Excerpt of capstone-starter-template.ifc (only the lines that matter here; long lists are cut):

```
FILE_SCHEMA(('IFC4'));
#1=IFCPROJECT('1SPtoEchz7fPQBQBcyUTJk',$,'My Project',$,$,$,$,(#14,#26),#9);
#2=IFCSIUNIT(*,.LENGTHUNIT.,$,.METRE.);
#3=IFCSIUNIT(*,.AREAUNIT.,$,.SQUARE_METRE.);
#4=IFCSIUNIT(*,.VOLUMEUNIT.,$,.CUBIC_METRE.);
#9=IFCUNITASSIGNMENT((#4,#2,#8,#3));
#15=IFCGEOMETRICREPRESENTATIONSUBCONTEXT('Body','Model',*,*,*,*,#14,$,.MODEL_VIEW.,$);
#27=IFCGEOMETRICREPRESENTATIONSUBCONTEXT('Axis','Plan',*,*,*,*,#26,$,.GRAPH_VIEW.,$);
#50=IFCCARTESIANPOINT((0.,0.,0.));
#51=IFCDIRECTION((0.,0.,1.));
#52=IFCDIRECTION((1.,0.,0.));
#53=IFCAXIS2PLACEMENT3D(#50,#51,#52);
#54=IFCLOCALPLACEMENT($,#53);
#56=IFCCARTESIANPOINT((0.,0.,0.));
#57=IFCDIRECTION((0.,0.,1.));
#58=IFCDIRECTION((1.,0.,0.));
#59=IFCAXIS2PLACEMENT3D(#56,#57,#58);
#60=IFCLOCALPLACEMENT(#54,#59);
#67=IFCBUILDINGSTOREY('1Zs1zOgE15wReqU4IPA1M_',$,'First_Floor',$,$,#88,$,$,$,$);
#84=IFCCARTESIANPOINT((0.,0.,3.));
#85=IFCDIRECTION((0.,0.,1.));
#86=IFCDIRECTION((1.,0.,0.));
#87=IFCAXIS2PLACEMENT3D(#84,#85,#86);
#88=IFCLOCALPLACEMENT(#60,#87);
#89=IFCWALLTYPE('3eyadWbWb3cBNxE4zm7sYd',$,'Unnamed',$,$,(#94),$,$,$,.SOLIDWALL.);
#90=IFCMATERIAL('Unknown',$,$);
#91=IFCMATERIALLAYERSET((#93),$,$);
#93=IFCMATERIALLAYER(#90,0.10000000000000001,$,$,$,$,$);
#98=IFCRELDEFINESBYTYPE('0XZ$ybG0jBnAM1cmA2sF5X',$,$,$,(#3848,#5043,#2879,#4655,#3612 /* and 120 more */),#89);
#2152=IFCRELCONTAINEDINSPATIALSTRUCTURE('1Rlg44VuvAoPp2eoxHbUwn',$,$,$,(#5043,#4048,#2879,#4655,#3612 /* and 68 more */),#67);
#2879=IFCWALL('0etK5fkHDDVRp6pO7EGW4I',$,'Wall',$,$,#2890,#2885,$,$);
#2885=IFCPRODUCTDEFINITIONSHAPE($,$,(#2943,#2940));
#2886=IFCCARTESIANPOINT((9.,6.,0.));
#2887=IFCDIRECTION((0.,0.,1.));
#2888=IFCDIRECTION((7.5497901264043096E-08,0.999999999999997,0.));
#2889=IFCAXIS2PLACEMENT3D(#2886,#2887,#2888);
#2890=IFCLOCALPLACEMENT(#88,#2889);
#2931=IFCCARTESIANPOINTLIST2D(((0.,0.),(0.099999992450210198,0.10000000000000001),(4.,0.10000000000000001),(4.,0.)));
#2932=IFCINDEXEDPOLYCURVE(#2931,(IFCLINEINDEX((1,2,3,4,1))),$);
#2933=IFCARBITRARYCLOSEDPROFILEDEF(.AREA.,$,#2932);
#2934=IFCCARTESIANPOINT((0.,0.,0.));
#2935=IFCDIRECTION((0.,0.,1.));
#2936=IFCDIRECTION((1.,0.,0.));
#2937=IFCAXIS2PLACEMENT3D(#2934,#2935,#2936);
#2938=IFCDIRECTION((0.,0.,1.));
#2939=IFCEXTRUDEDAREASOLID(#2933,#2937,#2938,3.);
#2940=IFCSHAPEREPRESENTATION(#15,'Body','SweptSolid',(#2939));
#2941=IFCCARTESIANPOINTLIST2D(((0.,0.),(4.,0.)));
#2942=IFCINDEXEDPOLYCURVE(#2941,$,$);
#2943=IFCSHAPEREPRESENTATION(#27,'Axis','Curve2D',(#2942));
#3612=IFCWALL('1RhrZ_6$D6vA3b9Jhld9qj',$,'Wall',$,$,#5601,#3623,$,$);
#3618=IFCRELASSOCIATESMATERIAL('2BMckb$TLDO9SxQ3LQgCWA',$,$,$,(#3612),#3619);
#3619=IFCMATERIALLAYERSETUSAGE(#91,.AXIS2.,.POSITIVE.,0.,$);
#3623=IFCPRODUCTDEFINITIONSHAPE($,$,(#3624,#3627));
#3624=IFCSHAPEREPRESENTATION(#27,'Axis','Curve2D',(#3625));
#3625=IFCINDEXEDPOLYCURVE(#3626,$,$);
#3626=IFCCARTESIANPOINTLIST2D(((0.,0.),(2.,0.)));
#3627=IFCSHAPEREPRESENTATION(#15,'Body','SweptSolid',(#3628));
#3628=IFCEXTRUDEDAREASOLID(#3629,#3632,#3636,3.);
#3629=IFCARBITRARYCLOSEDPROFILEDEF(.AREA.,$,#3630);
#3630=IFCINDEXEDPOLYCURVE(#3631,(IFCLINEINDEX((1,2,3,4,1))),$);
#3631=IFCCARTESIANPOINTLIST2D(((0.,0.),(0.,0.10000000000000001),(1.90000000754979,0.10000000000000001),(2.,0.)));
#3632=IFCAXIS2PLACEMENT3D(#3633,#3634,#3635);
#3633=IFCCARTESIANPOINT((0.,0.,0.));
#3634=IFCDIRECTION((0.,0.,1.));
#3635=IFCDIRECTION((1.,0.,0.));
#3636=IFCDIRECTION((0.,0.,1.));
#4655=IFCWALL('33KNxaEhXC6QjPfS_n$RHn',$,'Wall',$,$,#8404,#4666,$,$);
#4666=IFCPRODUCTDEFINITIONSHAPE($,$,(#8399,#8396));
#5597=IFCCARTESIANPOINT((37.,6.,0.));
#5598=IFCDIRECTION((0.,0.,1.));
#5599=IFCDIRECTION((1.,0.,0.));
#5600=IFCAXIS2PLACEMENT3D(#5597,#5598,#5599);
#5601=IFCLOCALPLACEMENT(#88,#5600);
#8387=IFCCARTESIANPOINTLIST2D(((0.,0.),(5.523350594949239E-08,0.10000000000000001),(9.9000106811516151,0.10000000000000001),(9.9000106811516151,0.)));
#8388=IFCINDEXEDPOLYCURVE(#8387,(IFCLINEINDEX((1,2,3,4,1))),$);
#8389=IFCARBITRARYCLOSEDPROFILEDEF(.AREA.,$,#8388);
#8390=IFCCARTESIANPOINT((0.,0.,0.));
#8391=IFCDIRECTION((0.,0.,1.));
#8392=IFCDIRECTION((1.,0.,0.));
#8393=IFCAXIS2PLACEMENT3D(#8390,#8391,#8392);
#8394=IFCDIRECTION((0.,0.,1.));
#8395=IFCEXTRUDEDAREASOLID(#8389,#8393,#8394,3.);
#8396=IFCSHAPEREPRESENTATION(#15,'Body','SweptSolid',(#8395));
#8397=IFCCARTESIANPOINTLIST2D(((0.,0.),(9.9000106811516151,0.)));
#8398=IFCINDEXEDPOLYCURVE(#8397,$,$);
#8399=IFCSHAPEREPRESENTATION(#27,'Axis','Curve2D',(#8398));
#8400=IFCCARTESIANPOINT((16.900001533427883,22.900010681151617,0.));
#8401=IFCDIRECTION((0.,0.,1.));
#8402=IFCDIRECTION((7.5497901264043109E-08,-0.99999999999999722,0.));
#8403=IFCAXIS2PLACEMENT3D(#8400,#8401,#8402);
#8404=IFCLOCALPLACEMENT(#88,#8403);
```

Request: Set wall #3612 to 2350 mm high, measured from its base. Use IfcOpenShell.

```python
import ifcopenshell
import ifcopenshell.geom
import ifcopenshell.util.representation
import ifcopenshell.util.shape
import ifcopenshell.util.unit

model = ifcopenshell.open("capstone-starter-template.ifc")
unit_scale = ifcopenshell.util.unit.calculate_unit_scale(model)
settings = ifcopenshell.geom.settings()


def volume(element):
    """Net volume in cubic metres, openings subtracted."""
    shape = ifcopenshell.geom.create_shape(settings, element)
    return ifcopenshell.util.shape.get_volume(shape.geometry)


wall = model.by_guid("1RhrZ_6$D6vA3b9Jhld9qj")
before = volume(wall)

body = ifcopenshell.util.representation.get_representation(wall, "Model", "Body")
solid = body.Items[0]
old_height = solid.Depth
solid.Depth = 2.35 / unit_scale
after = volume(wall)

print(f"height {old_height:g} -> {solid.Depth:g}, volume {before:.3f} -> {after:.3f} m3")

model.write("capstone-starter-template_edited.ifc")
```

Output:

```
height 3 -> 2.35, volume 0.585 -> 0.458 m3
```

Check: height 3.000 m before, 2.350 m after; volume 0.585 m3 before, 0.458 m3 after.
